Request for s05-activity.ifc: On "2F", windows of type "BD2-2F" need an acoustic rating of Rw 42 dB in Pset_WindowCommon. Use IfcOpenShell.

First a look at what the model holds.

```python
import ifcopenshell
import ifcopenshell.util.element

model = ifcopenshell.open("s05-activity.ifc")
print(model.schema)
storey = next(s for s in model.by_type("IfcBuildingStorey") if s.Name == "2F")
windows = [e for e in ifcopenshell.util.element.get_decomposition(storey) if e.is_a("IfcWindow")]
seen = {}
for e in windows:
    element_type = ifcopenshell.util.element.get_type(e)
    key = (element_type.Name if element_type != e and element_type else None, ifcopenshell.util.element.get_pset(e, "Pset_WindowCommon", "AcousticRating"))
    seen[key] = seen.get(key, 0) + 1
for (name, value), count in sorted(seen.items(), key=str):
    print(count, "x", name, "|", value)
```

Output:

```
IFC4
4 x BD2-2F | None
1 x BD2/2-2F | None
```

```python
import ifcopenshell
import ifcopenshell.api.pset
import ifcopenshell.util.element

model = ifcopenshell.open("s05-activity.ifc")

storey = next(s for s in model.by_type("IfcBuildingStorey") if s.Name == "2F")
windows = [e for e in ifcopenshell.util.element.get_decomposition(storey) if e.is_a("IfcWindow")]

count = 0
for e in windows:
    element_type = ifcopenshell.util.element.get_type(e)
    if element_type in (None, e) or element_type.Name != "BD2-2F":
        continue
    # add_pset returns the element's existing set when there is one.
    pset = ifcopenshell.api.pset.add_pset(model, product=e, name="Pset_WindowCommon")
    ifcopenshell.api.pset.edit_pset(model, pset=pset, properties={"AcousticRating": "Rw 42 dB"})
    count += 1

print(count, "windows updated")

model.write("s05-activity_edited.ifc")
```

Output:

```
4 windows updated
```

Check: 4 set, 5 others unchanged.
